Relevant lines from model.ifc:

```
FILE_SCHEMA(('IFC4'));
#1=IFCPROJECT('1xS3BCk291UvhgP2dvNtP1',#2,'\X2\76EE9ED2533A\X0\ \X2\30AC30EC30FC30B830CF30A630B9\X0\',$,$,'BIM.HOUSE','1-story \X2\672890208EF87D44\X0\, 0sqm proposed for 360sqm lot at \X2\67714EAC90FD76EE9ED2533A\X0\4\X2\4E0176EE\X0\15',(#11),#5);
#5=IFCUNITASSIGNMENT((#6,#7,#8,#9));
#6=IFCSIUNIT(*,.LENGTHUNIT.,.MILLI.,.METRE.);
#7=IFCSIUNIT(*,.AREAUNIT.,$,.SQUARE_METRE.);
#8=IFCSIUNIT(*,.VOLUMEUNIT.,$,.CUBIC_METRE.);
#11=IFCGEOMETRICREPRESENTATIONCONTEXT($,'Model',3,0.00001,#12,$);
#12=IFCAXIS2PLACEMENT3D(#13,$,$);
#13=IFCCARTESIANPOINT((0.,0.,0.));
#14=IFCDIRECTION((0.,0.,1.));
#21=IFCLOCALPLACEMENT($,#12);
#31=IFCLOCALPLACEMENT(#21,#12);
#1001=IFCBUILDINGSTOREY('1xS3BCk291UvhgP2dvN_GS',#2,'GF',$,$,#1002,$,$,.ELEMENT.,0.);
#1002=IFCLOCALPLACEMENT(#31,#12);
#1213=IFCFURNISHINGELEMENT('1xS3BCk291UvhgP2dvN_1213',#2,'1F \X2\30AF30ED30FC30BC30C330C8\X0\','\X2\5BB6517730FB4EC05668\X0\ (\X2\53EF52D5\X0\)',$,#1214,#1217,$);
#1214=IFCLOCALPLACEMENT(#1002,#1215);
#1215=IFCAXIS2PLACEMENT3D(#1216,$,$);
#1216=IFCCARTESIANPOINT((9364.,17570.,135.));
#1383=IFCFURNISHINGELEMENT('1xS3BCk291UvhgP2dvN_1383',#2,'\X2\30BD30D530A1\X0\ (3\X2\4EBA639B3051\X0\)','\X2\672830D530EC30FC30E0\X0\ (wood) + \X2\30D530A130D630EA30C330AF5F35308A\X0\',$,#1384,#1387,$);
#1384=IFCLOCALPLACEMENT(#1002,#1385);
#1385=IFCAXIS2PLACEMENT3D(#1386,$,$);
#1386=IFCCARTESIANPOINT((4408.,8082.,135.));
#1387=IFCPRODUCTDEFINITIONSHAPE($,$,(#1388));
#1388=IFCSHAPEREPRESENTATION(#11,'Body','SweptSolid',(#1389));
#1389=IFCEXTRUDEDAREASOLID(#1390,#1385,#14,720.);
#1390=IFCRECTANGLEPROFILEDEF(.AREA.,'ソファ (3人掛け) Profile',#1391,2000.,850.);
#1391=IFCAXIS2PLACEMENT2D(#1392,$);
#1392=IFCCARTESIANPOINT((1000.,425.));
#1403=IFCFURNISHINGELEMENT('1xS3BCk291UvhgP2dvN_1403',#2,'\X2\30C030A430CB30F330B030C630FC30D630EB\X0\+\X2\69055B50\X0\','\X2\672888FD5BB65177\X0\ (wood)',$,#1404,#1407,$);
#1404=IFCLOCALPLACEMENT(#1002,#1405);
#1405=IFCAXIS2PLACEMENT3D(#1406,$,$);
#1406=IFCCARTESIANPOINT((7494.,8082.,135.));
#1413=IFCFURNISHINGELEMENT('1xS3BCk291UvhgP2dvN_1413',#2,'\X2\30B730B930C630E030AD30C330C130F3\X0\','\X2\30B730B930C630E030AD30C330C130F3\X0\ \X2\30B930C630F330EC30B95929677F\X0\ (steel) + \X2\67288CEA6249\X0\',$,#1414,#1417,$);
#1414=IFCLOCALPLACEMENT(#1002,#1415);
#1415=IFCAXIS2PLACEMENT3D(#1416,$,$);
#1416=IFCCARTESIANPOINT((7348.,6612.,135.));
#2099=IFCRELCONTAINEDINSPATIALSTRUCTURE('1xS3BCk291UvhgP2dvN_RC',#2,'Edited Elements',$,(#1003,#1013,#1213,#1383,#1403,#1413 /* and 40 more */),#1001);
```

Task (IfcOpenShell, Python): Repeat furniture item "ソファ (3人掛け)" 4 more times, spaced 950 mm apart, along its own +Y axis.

```python
import ifcopenshell
import ifcopenshell.api.geometry
import ifcopenshell.api.root
import ifcopenshell.util.element
import ifcopenshell.util.placement
import ifcopenshell.util.unit

model = ifcopenshell.open("model.ifc")
unit_scale = ifcopenshell.util.unit.calculate_unit_scale(model)


def reuse_history(source, copy):
    """copy_class also copies each property set's owner history, people and application; keep the originals."""
    for rel in copy.IsDefinedBy:
        if rel.is_a("IfcRelDefinesByProperties") and (history := rel.RelatingPropertyDefinition.OwnerHistory):
            rel.RelatingPropertyDefinition.OwnerHistory = source.OwnerHistory
            ifcopenshell.util.element.remove_deep2(model, history)


source = model.by_guid("1xS3BCk291UvhgP2dvN_1383")
base = ifcopenshell.util.placement.get_local_placement(source.ObjectPlacement)
step = base[:3, 1] * 0.95 / unit_scale

for i in range(1, 5):
    copy = ifcopenshell.api.root.copy_class(model, product=source)
    copy.Representation = ifcopenshell.util.element.copy_deep(
        model, source.Representation, exclude=["IfcGeometricRepresentationContext", "IfcRepresentationMap"]
    )
    reuse_history(source, copy)
    matrix = base.copy()
    matrix[:3, 3] += i * step
    print("added at", matrix[:3, 3].round(3) + 0.0)
    ifcopenshell.api.geometry.edit_object_placement(model, product=copy, matrix=matrix, is_si=False)

model.write("model-out.ifc")
```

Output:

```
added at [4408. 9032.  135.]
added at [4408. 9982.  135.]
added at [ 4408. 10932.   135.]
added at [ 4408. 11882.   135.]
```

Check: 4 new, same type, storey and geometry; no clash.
